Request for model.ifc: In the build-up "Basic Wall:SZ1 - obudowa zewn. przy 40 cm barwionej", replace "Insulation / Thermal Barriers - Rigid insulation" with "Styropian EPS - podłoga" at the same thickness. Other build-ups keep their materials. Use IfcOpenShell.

First a look at what the model holds.

```python
import ifcopenshell
import ifcopenshell.util.element

model = ifcopenshell.open("model.ifc")
print(model.schema)
for layer_set in model.by_type("IfcMaterialLayerSet"):
    if layer_set.LayerSetName == "Basic Wall:SZ1 - obudowa zewn. przy 40 cm barwionej":
        for layer in layer_set.MaterialLayers:
            print(layer.id(), layer.Material and layer.Material.Name, layer.LayerThickness, sep=" | ")
        print(len(ifcopenshell.util.element.get_elements_by_material(model, layer_set)), "elements and types use it")
print(sorted(m.Name for m in model.by_type("IfcMaterial") if m.Name)[:60])
```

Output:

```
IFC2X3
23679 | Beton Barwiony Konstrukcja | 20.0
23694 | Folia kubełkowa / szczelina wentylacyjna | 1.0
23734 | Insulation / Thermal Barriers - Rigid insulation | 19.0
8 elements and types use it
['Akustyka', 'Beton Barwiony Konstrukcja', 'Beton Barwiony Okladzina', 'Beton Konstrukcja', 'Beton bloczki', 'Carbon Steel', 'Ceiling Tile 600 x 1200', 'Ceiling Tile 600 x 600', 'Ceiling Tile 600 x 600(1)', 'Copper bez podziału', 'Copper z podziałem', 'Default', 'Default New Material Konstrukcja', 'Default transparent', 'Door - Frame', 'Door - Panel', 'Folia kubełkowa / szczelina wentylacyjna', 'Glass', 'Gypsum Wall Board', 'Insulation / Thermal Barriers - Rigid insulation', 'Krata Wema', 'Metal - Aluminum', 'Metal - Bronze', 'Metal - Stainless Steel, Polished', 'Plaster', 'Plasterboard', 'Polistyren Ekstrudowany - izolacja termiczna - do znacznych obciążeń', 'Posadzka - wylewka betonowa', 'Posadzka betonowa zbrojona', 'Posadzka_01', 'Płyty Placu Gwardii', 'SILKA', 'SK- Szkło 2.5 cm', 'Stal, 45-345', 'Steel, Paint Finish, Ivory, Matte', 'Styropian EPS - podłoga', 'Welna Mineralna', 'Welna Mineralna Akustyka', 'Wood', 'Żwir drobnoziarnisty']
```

```python
import ifcopenshell
import ifcopenshell.api.material

model = ifcopenshell.open("model.ifc")

layer_set = next(s for s in model.by_type("IfcMaterialLayerSet") if s.LayerSetName == "Basic Wall:SZ1 - obudowa zewn. przy 40 cm barwionej")
layer = next(l for l in layer_set.MaterialLayers if l.Material and l.Material.Name == "Insulation / Thermal Barriers - Rigid insulation")
material = next(m for m in model.by_type("IfcMaterial") if m.Name == "Styropian EPS - podłoga")

# Point this one layer at the other material; renaming the old one would change it everywhere.
ifcopenshell.api.material.edit_layer(model, layer=layer, attributes={}, material=material)

print([l.Material.Name if l.Material else None for l in layer_set.MaterialLayers])

model.write("model_rev.ifc")
```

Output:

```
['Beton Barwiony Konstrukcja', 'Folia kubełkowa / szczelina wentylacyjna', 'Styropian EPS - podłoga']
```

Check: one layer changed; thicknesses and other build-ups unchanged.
